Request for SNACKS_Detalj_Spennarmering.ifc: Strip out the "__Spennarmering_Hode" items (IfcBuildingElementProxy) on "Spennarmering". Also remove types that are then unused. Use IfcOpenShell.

First a look at what the model holds.

```python
import ifcopenshell
import ifcopenshell.util.element

model = ifcopenshell.open("SNACKS_Detalj_Spennarmering.ifc")
print(model.schema)
storey = next(s for s in model.by_type("IfcBuildingStorey") if s.Name == "Spennarmering")
proxies = [e for e in ifcopenshell.util.element.get_decomposition(storey) if e.is_a("IfcBuildingElementProxy")]
seen = {}
for e in proxies:
    element_type = ifcopenshell.util.element.get_type(e)
    name = element_type.Name if element_type not in (None, e) else None
    seen[name] = seen.get(name, 0) + 1
for name, count in sorted(seen.items(), key=str):
    print(count, "x", name)
```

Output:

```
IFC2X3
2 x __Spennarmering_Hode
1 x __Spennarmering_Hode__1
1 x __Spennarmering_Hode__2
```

```python
import ifcopenshell
import ifcopenshell.api.root
import ifcopenshell.util.element

model = ifcopenshell.open("SNACKS_Detalj_Spennarmering.ifc")

storey = next(s for s in model.by_type("IfcBuildingStorey") if s.Name == "Spennarmering")
proxies = [e for e in ifcopenshell.util.element.get_decomposition(storey) if e.is_a("IfcBuildingElementProxy")]
targets = [e for e in proxies if (t := ifcopenshell.util.element.get_type(e)) not in (None, e) and t.Name == "__Spennarmering_Hode"]
types = {ifcopenshell.util.element.get_type(e) for e in targets} - {None, *targets}

for e in targets:
    ifcopenshell.api.root.remove_product(model, product=e)
print(len(targets), "removed")

unused = [t for t in types if not ifcopenshell.util.element.get_types(t)]
for t in unused:
    ifcopenshell.api.root.remove_product(model, product=t)
print(len(unused), "unused types removed")

model.write("SNACKS_Detalj_Spennarmering_rev.ifc")
```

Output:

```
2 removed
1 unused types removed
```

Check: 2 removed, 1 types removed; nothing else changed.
